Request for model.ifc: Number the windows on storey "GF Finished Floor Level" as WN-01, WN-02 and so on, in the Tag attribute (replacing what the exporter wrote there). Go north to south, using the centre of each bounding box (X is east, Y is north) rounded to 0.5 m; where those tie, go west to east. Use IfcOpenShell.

First a look at what the model holds.

```python
import ifcopenshell
import ifcopenshell.util.element
import ifcopenshell.util.placement

model = ifcopenshell.open("model.ifc")
print(model.schema)
storey = next(s for s in model.by_type("IfcBuildingStorey") if s.Name == "GF Finished Floor Level")
windows = [e for e in ifcopenshell.util.element.get_decomposition(storey) if e.is_a("IfcWindow")]
for e in sorted(windows, key=lambda e: e.id()):
    origin = ifcopenshell.util.placement.get_local_placement(e.ObjectPlacement)[:3, 3]
    print(e.id(), e.Tag, e.Name, origin.round(2) + 0.0, sep=" | ")
```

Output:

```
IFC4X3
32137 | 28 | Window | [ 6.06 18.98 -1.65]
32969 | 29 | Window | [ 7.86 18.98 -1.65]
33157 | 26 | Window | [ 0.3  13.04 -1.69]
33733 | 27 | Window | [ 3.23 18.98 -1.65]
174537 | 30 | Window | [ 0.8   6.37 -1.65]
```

```python
import ifcopenshell
import ifcopenshell.geom
import ifcopenshell.util.element
import ifcopenshell.util.shape

model = ifcopenshell.open("model.ifc")
settings = ifcopenshell.geom.settings()
settings.set("use-world-coords", True)


def centre(element):
    shape = ifcopenshell.geom.create_shape(settings, element)
    return ifcopenshell.util.shape.get_bbox_centroid(shape.geometry)


storey = next(s for s in model.by_type("IfcBuildingStorey") if s.Name == "GF Finished Floor Level")
windows = [e for e in ifcopenshell.util.element.get_decomposition(storey) if e.is_a("IfcWindow")]

# Insertion points can sit at a corner or the storey origin, so sort by the geometry (in metres).
centres = {e: centre(e) for e in windows}
windows.sort(key=lambda e: (-round(centres[e][1] / 0.5), centres[e][0]))

for i, e in enumerate(windows, start=1):
    number = f"WN-{i:02d}"
    e.Tag = number
    print(e.id(), number)

model.write("model_updated.ifc")
```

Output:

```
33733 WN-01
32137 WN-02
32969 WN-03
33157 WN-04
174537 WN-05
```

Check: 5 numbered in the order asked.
